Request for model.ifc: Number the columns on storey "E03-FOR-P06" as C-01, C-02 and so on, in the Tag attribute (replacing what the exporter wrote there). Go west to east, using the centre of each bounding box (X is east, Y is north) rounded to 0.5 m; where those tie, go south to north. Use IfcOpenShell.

First a look at what the model holds.

```python
import ifcopenshell
import ifcopenshell.util.element
import ifcopenshell.util.placement

model = ifcopenshell.open("model.ifc")
print(model.schema)
storey = next(s for s in model.by_type("IfcBuildingStorey") if s.Name == "E03-FOR-P06")
columns = [e for e in ifcopenshell.util.element.get_decomposition(storey) if e.is_a("IfcColumn")]
for e in sorted(columns, key=lambda e: e.id()):
    origin = ifcopenshell.util.placement.get_local_placement(e.ObjectPlacement)[:3, 3]
    print(e.id(), e.Tag, e.Name, origin.round(2) + 0.0, sep=" | ")
```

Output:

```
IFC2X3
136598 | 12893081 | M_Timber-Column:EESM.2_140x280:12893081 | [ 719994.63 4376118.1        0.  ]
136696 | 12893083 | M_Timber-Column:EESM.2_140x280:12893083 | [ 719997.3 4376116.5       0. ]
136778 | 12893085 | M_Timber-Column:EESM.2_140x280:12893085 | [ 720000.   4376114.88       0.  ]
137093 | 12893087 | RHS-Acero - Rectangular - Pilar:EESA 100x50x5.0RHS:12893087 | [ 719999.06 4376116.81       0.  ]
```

```python
import ifcopenshell
import ifcopenshell.geom
import ifcopenshell.util.element
import ifcopenshell.util.shape

model = ifcopenshell.open("model.ifc")
settings = ifcopenshell.geom.settings()
settings.set("use-world-coords", True)


def centre(element):
    shape = ifcopenshell.geom.create_shape(settings, element)
    return ifcopenshell.util.shape.get_bbox_centroid(shape.geometry)


storey = next(s for s in model.by_type("IfcBuildingStorey") if s.Name == "E03-FOR-P06")
columns = [e for e in ifcopenshell.util.element.get_decomposition(storey) if e.is_a("IfcColumn")]

# Insertion points can sit at a corner or the storey origin, so sort by the geometry (in metres).
centres = {e: centre(e) for e in columns}
columns.sort(key=lambda e: (round(centres[e][0] / 0.5), centres[e][1]))

for i, e in enumerate(columns, start=1):
    number = f"C-{i:02d}"
    e.Tag = number
    print(e.id(), number)

model.write("model_rev.ifc")
```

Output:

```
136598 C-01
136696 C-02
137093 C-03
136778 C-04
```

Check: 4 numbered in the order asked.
